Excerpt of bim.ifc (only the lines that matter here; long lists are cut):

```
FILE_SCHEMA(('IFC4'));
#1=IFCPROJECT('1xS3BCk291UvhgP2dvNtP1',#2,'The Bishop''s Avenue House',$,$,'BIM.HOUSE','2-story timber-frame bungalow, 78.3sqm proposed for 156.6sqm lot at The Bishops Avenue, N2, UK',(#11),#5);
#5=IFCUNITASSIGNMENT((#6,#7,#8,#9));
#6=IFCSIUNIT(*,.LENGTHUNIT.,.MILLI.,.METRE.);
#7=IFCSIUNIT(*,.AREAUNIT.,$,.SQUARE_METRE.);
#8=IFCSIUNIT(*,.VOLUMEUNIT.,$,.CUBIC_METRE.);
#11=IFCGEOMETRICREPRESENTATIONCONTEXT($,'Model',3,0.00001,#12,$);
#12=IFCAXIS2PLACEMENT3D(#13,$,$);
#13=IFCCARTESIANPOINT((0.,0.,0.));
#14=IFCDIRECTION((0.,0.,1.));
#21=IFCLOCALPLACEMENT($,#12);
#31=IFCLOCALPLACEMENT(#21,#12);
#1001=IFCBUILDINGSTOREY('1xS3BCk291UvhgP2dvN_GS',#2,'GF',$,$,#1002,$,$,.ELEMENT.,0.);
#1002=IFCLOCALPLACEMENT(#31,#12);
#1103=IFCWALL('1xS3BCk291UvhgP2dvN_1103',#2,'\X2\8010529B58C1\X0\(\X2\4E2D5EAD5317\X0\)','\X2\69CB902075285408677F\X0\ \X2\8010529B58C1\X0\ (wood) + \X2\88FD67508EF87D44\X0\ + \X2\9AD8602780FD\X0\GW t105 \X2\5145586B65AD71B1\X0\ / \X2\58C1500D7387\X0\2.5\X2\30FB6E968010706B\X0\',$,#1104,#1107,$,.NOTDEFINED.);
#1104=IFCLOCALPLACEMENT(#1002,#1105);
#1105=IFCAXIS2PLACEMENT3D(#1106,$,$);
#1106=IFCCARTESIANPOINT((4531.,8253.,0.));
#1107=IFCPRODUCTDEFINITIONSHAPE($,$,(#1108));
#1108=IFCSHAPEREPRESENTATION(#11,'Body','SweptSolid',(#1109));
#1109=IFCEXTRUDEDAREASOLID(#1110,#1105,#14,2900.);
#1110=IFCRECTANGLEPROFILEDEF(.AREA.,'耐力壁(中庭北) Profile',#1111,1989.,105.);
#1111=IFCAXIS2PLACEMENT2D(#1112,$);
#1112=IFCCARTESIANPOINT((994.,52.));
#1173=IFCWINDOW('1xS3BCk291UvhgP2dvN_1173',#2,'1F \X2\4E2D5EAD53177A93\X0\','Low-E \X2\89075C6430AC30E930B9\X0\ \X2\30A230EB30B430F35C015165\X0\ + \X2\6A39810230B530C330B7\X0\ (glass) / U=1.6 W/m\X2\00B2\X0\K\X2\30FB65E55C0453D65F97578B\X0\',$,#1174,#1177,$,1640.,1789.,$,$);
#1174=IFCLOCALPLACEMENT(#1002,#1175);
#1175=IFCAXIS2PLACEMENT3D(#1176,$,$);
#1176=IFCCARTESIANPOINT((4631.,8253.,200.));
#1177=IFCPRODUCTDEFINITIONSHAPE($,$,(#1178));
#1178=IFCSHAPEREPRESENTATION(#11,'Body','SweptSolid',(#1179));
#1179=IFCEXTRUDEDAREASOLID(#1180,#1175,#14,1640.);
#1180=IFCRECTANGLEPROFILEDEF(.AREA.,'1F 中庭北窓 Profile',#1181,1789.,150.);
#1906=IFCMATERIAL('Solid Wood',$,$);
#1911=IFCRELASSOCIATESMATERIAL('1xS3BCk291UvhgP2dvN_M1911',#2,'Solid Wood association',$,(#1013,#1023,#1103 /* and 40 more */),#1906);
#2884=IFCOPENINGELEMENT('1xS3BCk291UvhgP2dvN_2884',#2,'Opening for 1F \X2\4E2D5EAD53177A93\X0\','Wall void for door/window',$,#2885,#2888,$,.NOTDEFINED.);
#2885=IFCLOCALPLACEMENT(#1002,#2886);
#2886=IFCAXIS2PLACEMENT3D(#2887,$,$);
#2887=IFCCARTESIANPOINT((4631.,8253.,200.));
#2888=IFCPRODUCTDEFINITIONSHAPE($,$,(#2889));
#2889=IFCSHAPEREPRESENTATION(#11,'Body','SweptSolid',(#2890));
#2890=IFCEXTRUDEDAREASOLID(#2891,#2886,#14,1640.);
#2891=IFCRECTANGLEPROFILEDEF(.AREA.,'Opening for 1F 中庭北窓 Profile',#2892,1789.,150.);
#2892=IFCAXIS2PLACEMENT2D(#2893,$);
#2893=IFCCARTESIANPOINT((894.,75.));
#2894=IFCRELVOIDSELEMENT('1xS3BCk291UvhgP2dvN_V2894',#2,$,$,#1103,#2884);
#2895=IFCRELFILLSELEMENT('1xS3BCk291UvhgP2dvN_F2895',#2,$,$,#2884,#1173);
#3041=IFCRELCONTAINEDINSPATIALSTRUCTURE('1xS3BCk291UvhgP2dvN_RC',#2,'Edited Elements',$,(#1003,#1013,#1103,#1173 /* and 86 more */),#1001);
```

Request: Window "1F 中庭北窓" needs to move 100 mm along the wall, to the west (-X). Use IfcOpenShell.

```python
import ifcopenshell
import ifcopenshell.api.geometry
import ifcopenshell.util.placement

model = ifcopenshell.open("bim.ifc")

window = model.by_id(1173)
opening = window.FillsVoids[0].RelatingOpeningElement
wall = opening.VoidsElements[0].RelatingBuildingElement

wall_matrix = ifcopenshell.util.placement.get_local_placement(wall.ObjectPlacement)
shift = wall_matrix[:3, 0] * -100.0
before = ifcopenshell.util.placement.get_local_placement(window.ObjectPlacement)[:3, 3].copy()

# The window is not placed relative to its opening, so move both.
for product in (opening, window):
    matrix = ifcopenshell.util.placement.get_local_placement(product.ObjectPlacement)
    matrix[:3, 3] += shift
    ifcopenshell.api.geometry.edit_object_placement(model, product=product, matrix=matrix, is_si=False)

after = ifcopenshell.util.placement.get_local_placement(window.ObjectPlacement)[:3, 3]
print("window moved by", (after - before).round(3) + 0.0)

model.write("bim_rev.ifc")
```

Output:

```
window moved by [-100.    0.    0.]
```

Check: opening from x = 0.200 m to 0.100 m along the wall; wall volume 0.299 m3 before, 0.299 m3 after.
